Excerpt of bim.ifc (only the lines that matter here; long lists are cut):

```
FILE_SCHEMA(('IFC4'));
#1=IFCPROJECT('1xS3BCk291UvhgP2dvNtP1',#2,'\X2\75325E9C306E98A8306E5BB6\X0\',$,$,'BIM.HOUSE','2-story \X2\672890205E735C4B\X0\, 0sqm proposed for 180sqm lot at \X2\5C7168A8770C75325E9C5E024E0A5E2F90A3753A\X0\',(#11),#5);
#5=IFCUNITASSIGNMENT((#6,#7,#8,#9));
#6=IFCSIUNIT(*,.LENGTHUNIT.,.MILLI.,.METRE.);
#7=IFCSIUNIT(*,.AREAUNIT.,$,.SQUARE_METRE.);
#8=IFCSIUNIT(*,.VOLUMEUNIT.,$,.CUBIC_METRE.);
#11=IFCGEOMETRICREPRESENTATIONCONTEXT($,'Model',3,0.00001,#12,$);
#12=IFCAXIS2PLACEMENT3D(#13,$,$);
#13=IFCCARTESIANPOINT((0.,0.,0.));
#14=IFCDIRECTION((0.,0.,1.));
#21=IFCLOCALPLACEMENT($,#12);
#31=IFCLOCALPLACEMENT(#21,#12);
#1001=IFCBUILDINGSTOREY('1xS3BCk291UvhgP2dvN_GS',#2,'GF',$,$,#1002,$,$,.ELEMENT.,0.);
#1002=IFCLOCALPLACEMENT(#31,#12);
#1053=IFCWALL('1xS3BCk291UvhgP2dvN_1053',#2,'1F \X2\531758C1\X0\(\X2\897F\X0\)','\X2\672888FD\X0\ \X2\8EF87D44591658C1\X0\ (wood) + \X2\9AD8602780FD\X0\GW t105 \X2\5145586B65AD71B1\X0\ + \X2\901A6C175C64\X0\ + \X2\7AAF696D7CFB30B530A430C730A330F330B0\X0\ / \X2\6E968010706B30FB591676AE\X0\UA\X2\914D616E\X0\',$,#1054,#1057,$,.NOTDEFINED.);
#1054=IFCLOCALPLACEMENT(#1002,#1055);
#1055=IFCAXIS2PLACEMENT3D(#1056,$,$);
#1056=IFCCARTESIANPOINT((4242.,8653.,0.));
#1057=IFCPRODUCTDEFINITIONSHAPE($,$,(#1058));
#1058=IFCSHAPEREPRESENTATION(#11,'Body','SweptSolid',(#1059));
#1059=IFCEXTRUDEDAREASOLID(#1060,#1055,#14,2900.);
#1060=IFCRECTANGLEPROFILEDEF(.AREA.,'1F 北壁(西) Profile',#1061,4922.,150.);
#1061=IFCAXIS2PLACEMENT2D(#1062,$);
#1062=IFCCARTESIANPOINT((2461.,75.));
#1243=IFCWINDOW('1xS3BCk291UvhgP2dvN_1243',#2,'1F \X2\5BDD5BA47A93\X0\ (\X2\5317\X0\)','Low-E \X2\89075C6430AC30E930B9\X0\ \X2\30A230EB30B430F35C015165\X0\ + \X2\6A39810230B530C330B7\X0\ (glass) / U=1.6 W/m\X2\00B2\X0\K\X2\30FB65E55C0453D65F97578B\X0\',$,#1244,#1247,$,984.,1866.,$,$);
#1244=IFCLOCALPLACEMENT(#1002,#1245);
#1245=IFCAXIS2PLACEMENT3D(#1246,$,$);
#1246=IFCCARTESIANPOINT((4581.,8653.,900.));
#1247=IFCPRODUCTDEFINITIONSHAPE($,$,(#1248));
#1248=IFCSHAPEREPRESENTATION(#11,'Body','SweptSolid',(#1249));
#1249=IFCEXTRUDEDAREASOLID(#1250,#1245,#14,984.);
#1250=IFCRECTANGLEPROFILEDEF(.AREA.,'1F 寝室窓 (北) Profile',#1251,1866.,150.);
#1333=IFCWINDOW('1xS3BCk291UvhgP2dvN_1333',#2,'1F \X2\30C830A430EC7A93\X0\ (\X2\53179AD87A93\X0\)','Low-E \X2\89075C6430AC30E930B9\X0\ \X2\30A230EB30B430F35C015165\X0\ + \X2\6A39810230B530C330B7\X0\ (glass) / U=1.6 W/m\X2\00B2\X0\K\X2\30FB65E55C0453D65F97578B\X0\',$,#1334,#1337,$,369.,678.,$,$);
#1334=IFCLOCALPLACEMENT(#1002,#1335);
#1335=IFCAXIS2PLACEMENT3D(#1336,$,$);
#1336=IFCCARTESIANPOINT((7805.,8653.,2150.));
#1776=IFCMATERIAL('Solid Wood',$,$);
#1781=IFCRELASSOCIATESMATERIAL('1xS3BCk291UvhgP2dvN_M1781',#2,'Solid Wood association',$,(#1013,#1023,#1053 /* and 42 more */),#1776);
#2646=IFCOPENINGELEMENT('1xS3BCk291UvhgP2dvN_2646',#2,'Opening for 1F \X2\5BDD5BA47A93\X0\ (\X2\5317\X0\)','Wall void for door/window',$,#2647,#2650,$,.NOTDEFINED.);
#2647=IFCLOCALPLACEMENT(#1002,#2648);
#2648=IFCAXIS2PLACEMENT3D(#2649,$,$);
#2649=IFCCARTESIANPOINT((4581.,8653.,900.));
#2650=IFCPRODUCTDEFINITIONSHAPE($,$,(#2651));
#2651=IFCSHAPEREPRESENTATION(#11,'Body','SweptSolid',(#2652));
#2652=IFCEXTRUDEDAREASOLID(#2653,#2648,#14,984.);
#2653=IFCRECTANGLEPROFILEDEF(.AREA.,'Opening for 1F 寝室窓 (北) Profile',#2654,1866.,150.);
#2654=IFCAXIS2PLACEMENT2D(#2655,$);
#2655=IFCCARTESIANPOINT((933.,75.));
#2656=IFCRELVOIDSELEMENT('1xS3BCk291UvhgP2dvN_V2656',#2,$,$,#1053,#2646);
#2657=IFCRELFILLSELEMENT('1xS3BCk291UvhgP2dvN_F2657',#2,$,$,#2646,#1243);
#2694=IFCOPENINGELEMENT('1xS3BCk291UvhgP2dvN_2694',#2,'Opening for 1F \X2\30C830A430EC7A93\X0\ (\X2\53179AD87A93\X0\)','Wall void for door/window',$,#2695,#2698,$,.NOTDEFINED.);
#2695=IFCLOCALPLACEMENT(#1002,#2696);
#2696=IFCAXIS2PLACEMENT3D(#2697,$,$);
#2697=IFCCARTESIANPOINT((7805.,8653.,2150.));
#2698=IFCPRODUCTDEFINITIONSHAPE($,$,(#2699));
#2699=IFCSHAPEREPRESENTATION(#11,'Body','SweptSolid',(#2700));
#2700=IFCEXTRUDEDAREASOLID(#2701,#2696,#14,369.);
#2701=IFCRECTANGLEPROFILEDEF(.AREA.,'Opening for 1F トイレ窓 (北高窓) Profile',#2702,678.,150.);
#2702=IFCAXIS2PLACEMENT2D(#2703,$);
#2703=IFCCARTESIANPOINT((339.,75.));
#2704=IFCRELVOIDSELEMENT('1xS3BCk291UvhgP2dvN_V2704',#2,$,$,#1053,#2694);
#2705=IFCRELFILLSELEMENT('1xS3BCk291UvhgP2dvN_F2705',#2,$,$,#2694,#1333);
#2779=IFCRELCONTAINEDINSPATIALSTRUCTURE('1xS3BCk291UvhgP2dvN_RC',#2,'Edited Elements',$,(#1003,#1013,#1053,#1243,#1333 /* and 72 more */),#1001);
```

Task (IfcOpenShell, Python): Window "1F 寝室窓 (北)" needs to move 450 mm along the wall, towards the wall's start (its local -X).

```python
import ifcopenshell
import ifcopenshell.api.geometry
import ifcopenshell.util.placement
import ifcopenshell.util.unit

model = ifcopenshell.open("bim.ifc")
unit_scale = ifcopenshell.util.unit.calculate_unit_scale(model)

window = model.by_id(1243)
opening = window.FillsVoids[0].RelatingOpeningElement
wall = opening.VoidsElements[0].RelatingBuildingElement

wall_matrix = ifcopenshell.util.placement.get_local_placement(wall.ObjectPlacement)
shift = wall_matrix[:3, 0] * -0.45 / unit_scale
before = ifcopenshell.util.placement.get_local_placement(window.ObjectPlacement)[:3, 3].copy()

# The window is not placed relative to its opening, so move both.
for product in (opening, window):
    matrix = ifcopenshell.util.placement.get_local_placement(product.ObjectPlacement)
    matrix[:3, 3] += shift
    ifcopenshell.api.geometry.edit_object_placement(model, product=product, matrix=matrix, is_si=False)

after = ifcopenshell.util.placement.get_local_placement(window.ObjectPlacement)[:3, 3]
print("window moved by", (after - before).round(3) + 0.0)

model.write("bim_rev.ifc")
```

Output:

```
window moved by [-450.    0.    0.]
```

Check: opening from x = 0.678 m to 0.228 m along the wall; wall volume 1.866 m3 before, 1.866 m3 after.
